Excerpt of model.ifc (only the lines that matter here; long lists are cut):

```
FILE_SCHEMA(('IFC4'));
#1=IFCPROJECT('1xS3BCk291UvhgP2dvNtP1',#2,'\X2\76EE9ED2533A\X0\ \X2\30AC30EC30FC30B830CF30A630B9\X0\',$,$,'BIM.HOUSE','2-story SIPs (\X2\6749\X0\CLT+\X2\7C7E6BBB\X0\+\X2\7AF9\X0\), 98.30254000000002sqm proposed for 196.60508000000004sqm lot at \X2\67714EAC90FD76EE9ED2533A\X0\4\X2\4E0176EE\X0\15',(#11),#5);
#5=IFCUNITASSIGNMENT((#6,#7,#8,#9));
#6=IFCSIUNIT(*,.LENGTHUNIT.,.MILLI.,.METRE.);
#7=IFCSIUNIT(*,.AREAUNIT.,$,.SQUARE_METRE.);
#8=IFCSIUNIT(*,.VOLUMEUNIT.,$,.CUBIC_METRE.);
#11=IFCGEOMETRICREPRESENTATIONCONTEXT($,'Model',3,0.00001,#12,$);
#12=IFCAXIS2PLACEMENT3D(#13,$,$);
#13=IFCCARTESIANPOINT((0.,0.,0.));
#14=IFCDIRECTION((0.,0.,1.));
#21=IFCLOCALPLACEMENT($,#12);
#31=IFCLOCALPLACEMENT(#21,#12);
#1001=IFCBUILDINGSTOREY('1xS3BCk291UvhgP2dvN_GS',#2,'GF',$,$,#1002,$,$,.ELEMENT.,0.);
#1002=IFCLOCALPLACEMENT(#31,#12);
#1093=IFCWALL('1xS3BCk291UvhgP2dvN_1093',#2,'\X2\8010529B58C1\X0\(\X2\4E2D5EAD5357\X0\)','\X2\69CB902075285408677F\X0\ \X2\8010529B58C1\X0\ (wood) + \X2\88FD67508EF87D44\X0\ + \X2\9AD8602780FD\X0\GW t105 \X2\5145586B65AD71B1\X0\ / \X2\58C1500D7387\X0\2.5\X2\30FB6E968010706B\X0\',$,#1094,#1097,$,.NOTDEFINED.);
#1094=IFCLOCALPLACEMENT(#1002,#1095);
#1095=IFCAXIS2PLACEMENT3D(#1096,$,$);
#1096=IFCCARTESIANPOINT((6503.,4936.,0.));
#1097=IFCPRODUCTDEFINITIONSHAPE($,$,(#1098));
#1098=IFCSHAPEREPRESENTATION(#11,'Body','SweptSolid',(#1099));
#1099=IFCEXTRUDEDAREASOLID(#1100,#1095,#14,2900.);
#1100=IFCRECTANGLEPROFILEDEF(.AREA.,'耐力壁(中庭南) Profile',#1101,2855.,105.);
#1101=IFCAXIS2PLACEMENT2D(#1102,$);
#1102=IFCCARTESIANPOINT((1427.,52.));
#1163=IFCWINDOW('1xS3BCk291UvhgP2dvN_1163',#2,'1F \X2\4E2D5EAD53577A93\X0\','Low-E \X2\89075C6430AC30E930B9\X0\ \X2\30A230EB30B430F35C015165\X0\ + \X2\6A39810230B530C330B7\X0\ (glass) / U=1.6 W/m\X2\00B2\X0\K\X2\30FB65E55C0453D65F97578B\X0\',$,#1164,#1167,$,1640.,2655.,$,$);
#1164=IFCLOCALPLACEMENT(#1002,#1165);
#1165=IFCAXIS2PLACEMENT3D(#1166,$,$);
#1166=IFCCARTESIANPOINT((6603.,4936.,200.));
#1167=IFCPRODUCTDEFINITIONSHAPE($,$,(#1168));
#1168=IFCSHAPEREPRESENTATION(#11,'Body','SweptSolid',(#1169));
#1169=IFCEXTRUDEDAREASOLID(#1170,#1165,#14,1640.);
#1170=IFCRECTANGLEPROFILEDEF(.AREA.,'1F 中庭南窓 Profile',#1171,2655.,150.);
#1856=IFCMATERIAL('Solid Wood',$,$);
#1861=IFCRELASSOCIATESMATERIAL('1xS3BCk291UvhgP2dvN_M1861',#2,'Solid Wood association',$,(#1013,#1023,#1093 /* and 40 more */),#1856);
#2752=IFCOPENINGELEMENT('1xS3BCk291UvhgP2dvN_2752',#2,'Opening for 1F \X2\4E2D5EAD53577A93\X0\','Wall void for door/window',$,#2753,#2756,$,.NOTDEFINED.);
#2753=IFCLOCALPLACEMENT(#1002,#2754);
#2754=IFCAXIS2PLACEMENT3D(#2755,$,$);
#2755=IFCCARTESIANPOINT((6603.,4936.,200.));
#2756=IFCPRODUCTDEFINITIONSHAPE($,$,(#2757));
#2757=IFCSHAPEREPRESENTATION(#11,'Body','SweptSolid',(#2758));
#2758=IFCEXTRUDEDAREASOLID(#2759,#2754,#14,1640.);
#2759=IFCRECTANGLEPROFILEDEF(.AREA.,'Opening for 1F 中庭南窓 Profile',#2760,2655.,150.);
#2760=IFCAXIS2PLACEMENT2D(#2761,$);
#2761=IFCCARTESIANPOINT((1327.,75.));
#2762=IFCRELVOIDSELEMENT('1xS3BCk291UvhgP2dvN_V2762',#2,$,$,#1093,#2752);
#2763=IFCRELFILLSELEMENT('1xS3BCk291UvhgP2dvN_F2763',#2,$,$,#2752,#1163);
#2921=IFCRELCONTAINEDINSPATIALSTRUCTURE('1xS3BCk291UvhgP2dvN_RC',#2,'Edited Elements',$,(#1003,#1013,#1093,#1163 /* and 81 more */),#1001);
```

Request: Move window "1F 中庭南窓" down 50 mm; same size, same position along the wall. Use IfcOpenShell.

```python
import numpy as np
import ifcopenshell
import ifcopenshell.api.geometry
import ifcopenshell.util.placement
import ifcopenshell.util.unit

model = ifcopenshell.open("model.ifc")
unit_scale = ifcopenshell.util.unit.calculate_unit_scale(model)

window = model.by_guid("1xS3BCk291UvhgP2dvN_1163")
opening = window.FillsVoids[0].RelatingOpeningElement
dz = -0.05 / unit_scale

shift = np.array([0.0, 0.0, dz])
# The window is not placed relative to its opening, so move both.
for product in (opening, window):
    matrix = ifcopenshell.util.placement.get_local_placement(product.ObjectPlacement)
    matrix[:3, 3] += shift
    ifcopenshell.api.geometry.edit_object_placement(model, product=product, matrix=matrix, is_si=False)

print(f"moved by {dz * unit_scale:+.3f} m")

model.write("model-out.ifc")
```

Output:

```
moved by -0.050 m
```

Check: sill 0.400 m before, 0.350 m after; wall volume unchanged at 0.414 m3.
